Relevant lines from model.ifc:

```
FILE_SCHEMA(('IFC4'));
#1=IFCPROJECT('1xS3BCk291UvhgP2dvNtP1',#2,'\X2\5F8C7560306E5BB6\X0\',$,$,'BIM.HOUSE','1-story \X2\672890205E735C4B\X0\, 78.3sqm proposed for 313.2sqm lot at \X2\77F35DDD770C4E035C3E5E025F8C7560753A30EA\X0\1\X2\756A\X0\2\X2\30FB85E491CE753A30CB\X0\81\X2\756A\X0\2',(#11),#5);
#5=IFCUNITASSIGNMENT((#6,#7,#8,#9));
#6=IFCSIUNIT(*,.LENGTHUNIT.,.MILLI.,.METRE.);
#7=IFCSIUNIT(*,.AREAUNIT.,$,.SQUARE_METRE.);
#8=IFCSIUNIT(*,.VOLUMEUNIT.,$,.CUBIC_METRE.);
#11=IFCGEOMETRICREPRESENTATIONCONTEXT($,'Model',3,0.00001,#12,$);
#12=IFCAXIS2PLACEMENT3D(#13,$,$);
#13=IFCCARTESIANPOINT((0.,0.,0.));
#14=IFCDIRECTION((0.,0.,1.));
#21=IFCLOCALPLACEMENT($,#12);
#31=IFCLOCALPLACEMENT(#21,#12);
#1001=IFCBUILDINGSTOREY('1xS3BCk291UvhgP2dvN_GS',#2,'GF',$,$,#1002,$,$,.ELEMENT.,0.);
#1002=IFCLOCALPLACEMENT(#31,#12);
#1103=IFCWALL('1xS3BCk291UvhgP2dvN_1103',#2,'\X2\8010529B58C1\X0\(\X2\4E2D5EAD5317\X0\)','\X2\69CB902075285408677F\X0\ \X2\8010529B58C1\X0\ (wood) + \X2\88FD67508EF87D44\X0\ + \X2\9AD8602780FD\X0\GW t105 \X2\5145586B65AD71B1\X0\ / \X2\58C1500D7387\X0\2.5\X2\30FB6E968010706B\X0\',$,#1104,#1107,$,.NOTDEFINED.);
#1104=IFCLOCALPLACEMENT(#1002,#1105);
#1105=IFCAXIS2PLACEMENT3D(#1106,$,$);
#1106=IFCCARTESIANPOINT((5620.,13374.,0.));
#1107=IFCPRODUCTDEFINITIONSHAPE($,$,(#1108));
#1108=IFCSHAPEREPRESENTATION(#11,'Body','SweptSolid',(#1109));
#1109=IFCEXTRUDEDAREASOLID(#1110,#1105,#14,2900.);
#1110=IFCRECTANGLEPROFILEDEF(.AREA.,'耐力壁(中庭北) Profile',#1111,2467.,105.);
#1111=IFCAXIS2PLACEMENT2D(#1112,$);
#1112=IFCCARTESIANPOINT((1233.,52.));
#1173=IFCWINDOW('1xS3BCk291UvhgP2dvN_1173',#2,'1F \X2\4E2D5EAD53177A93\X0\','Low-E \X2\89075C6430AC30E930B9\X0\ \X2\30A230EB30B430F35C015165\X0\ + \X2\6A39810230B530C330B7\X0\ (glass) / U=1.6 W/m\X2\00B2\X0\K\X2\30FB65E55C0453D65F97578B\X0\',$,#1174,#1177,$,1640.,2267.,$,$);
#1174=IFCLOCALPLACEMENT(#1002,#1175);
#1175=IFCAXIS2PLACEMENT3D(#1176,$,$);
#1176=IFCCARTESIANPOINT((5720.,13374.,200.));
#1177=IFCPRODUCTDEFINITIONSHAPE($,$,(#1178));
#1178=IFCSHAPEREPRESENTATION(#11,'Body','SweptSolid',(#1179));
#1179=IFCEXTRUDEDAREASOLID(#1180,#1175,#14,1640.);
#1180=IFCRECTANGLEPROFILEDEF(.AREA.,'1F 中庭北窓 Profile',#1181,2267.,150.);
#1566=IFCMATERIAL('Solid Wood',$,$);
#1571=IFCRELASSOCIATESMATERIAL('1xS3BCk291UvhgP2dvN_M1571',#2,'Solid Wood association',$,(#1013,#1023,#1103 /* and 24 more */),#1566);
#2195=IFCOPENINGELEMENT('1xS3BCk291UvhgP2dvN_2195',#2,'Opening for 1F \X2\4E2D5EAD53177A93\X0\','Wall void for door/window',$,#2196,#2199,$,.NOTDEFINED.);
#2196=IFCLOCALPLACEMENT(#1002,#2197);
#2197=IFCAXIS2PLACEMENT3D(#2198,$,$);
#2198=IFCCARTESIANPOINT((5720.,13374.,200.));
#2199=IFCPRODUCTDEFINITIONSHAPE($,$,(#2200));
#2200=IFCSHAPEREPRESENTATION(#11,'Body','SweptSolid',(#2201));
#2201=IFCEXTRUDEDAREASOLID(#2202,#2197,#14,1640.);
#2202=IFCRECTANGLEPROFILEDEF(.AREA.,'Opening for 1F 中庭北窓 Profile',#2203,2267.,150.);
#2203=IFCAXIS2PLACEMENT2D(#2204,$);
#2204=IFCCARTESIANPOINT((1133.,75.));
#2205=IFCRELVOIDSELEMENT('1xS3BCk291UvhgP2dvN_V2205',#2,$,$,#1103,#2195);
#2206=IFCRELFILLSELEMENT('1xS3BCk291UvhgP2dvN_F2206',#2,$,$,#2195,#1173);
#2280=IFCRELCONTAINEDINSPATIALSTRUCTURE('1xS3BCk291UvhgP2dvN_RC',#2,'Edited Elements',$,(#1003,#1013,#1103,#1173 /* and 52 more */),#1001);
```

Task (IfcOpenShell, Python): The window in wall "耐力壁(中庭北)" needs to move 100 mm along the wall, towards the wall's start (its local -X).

```python
import ifcopenshell
import ifcopenshell.api.geometry
import ifcopenshell.util.placement

model = ifcopenshell.open("model.ifc")

window = model.by_guid("1xS3BCk291UvhgP2dvN_1173")
opening = window.FillsVoids[0].RelatingOpeningElement
wall = opening.VoidsElements[0].RelatingBuildingElement

wall_matrix = ifcopenshell.util.placement.get_local_placement(wall.ObjectPlacement)
shift = wall_matrix[:3, 0] * -100.0
before = ifcopenshell.util.placement.get_local_placement(window.ObjectPlacement)[:3, 3].copy()

# The window is not placed relative to its opening, so move both.
for product in (opening, window):
    matrix = ifcopenshell.util.placement.get_local_placement(product.ObjectPlacement)
    matrix[:3, 3] += shift
    ifcopenshell.api.geometry.edit_object_placement(model, product=product, matrix=matrix, is_si=False)

after = ifcopenshell.util.placement.get_local_placement(window.ObjectPlacement)[:3, 3]
print("window moved by", (after - before).round(3) + 0.0)

model.write("model_edited.ifc")
```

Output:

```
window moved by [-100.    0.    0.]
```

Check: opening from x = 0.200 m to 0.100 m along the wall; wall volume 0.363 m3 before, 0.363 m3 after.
